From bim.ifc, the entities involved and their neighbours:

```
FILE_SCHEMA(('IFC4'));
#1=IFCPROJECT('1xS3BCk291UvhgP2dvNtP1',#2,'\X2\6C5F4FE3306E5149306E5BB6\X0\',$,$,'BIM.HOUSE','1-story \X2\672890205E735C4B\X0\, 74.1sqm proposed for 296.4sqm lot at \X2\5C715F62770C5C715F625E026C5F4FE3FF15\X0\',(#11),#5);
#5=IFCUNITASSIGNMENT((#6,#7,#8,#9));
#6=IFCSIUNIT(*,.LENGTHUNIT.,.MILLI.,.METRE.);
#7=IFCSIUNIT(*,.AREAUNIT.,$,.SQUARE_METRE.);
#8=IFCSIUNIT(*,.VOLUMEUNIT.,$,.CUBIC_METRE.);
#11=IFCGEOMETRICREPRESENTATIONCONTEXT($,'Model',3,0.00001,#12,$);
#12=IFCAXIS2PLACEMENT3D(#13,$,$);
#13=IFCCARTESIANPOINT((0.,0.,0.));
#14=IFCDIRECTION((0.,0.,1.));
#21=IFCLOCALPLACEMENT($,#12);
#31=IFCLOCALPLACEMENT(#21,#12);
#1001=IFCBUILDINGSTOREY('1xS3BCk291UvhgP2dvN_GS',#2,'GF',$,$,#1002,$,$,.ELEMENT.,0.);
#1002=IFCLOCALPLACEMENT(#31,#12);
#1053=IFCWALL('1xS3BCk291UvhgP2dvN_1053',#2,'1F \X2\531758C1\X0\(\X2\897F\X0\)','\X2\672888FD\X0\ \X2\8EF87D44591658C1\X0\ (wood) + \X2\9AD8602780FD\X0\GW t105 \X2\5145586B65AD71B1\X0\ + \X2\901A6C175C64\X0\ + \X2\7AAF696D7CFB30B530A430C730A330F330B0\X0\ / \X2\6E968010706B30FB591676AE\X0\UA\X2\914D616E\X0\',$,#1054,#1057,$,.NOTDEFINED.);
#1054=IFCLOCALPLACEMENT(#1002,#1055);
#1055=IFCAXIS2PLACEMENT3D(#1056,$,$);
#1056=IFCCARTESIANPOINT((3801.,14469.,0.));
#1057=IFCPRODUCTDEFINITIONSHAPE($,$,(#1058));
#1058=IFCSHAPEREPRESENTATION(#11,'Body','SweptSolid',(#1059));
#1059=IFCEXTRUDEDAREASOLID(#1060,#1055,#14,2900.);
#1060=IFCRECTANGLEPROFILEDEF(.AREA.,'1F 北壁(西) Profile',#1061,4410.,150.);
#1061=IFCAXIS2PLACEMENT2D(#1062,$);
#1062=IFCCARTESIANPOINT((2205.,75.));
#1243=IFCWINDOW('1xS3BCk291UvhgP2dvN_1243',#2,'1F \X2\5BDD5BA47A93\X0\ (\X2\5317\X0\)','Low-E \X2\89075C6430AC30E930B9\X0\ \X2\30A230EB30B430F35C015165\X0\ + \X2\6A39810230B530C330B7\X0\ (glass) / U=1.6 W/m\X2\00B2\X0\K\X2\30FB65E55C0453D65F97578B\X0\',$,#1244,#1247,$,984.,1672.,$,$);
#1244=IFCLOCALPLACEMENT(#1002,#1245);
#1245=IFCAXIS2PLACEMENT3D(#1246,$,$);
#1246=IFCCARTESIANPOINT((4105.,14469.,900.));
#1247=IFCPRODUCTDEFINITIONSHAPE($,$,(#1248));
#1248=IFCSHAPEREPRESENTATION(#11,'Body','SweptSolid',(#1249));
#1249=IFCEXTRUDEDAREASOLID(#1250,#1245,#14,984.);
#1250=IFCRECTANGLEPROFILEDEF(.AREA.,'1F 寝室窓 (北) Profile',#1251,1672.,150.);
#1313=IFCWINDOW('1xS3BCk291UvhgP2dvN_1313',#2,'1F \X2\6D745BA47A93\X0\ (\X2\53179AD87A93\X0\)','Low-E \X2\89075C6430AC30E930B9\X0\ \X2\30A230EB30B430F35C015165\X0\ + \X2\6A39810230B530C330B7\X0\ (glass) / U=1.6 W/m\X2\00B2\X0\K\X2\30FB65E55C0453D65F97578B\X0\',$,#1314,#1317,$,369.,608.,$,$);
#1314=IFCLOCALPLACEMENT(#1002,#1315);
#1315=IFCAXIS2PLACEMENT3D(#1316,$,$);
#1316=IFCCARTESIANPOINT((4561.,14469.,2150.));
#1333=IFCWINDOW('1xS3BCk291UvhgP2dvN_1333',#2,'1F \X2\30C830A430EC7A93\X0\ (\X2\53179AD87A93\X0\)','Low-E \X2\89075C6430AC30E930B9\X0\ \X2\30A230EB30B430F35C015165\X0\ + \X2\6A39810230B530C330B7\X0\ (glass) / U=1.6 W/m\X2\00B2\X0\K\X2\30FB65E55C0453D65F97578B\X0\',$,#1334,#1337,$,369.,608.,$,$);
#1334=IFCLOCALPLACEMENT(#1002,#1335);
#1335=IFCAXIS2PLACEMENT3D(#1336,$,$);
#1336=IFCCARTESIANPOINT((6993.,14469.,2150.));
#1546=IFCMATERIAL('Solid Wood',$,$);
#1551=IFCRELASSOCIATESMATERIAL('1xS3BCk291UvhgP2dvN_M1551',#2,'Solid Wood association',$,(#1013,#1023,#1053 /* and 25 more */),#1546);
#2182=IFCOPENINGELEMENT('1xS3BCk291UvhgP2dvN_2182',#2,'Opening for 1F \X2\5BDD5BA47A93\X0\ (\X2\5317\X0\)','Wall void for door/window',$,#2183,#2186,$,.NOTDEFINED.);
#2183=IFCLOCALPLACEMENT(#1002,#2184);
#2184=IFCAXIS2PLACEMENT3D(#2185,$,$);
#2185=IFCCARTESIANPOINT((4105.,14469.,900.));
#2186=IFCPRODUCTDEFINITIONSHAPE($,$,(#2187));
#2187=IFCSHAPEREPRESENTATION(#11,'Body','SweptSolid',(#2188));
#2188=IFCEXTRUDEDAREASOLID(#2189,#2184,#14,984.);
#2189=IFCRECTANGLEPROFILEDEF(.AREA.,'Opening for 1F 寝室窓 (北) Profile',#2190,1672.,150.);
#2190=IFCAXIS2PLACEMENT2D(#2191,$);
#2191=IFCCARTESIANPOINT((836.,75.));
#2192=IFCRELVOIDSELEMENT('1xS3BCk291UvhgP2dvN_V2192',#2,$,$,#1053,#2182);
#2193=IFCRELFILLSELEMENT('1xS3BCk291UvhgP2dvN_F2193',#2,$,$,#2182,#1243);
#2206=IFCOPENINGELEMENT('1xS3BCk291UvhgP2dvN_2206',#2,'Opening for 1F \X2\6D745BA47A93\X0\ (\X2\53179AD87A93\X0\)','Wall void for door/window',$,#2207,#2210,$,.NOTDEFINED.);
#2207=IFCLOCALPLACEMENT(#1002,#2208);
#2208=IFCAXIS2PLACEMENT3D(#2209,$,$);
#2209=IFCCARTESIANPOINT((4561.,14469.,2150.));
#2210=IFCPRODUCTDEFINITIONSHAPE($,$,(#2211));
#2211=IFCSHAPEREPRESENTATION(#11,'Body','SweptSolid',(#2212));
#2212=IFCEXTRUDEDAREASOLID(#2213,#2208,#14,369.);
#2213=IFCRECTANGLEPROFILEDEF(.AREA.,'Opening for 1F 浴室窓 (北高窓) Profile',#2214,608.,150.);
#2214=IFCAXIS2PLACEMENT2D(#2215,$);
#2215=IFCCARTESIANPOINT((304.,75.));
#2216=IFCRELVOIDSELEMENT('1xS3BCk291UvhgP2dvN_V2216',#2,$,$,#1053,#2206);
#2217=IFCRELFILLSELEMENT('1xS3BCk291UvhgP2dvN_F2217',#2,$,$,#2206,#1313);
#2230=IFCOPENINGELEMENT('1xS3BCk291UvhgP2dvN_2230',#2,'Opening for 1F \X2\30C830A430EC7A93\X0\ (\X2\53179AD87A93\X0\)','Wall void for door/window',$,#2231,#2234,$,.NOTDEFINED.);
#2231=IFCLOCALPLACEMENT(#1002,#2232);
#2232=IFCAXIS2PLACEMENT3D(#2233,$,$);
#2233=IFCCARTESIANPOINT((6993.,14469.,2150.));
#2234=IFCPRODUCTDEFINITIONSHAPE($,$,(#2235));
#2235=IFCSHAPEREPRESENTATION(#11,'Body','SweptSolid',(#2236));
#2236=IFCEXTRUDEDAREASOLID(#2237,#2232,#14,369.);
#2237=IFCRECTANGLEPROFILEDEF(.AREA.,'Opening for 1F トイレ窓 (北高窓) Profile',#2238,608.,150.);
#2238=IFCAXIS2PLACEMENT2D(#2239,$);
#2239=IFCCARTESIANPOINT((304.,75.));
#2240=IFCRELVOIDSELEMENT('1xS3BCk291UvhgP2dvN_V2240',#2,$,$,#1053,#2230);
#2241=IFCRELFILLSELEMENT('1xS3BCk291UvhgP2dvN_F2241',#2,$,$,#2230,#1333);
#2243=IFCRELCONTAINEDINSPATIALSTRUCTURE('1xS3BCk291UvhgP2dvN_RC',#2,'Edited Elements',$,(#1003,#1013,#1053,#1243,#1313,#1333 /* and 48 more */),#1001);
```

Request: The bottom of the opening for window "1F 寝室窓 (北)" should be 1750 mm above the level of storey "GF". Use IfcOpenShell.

```python
import numpy as np
import ifcopenshell
import ifcopenshell.api.geometry
import ifcopenshell.geom
import ifcopenshell.util.element
import ifcopenshell.util.placement
import ifcopenshell.util.shape
import ifcopenshell.util.unit

model = ifcopenshell.open("bim.ifc")
unit_scale = ifcopenshell.util.unit.calculate_unit_scale(model)

window = model.by_guid("1xS3BCk291UvhgP2dvN_1243")
opening = window.FillsVoids[0].RelatingOpeningElement
storey = ifcopenshell.util.element.get_container(window, ifc_class="IfcBuildingStorey")
level = ifcopenshell.util.placement.get_local_placement(storey.ObjectPlacement)[2, 3]

# The opening's origin need not be at the sill, so measure its lowest point.
shape = ifcopenshell.geom.create_shape(ifcopenshell.geom.settings(), opening)
bottom = ifcopenshell.util.shape.get_shape_bottom_elevation(shape, shape.geometry) / unit_scale
dz = level + 1750.0 - bottom

shift = np.array([0.0, 0.0, dz])
# The window is not placed relative to its opening, so move both.
for product in (opening, window):
    matrix = ifcopenshell.util.placement.get_local_placement(product.ObjectPlacement)
    matrix[:3, 3] += shift
    ifcopenshell.api.geometry.edit_object_placement(model, product=product, matrix=matrix, is_si=False)

print(f"moved by {dz * unit_scale:+.3f} m")

model.write("bim_updated.ifc")
```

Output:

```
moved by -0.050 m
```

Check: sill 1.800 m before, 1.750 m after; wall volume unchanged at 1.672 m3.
